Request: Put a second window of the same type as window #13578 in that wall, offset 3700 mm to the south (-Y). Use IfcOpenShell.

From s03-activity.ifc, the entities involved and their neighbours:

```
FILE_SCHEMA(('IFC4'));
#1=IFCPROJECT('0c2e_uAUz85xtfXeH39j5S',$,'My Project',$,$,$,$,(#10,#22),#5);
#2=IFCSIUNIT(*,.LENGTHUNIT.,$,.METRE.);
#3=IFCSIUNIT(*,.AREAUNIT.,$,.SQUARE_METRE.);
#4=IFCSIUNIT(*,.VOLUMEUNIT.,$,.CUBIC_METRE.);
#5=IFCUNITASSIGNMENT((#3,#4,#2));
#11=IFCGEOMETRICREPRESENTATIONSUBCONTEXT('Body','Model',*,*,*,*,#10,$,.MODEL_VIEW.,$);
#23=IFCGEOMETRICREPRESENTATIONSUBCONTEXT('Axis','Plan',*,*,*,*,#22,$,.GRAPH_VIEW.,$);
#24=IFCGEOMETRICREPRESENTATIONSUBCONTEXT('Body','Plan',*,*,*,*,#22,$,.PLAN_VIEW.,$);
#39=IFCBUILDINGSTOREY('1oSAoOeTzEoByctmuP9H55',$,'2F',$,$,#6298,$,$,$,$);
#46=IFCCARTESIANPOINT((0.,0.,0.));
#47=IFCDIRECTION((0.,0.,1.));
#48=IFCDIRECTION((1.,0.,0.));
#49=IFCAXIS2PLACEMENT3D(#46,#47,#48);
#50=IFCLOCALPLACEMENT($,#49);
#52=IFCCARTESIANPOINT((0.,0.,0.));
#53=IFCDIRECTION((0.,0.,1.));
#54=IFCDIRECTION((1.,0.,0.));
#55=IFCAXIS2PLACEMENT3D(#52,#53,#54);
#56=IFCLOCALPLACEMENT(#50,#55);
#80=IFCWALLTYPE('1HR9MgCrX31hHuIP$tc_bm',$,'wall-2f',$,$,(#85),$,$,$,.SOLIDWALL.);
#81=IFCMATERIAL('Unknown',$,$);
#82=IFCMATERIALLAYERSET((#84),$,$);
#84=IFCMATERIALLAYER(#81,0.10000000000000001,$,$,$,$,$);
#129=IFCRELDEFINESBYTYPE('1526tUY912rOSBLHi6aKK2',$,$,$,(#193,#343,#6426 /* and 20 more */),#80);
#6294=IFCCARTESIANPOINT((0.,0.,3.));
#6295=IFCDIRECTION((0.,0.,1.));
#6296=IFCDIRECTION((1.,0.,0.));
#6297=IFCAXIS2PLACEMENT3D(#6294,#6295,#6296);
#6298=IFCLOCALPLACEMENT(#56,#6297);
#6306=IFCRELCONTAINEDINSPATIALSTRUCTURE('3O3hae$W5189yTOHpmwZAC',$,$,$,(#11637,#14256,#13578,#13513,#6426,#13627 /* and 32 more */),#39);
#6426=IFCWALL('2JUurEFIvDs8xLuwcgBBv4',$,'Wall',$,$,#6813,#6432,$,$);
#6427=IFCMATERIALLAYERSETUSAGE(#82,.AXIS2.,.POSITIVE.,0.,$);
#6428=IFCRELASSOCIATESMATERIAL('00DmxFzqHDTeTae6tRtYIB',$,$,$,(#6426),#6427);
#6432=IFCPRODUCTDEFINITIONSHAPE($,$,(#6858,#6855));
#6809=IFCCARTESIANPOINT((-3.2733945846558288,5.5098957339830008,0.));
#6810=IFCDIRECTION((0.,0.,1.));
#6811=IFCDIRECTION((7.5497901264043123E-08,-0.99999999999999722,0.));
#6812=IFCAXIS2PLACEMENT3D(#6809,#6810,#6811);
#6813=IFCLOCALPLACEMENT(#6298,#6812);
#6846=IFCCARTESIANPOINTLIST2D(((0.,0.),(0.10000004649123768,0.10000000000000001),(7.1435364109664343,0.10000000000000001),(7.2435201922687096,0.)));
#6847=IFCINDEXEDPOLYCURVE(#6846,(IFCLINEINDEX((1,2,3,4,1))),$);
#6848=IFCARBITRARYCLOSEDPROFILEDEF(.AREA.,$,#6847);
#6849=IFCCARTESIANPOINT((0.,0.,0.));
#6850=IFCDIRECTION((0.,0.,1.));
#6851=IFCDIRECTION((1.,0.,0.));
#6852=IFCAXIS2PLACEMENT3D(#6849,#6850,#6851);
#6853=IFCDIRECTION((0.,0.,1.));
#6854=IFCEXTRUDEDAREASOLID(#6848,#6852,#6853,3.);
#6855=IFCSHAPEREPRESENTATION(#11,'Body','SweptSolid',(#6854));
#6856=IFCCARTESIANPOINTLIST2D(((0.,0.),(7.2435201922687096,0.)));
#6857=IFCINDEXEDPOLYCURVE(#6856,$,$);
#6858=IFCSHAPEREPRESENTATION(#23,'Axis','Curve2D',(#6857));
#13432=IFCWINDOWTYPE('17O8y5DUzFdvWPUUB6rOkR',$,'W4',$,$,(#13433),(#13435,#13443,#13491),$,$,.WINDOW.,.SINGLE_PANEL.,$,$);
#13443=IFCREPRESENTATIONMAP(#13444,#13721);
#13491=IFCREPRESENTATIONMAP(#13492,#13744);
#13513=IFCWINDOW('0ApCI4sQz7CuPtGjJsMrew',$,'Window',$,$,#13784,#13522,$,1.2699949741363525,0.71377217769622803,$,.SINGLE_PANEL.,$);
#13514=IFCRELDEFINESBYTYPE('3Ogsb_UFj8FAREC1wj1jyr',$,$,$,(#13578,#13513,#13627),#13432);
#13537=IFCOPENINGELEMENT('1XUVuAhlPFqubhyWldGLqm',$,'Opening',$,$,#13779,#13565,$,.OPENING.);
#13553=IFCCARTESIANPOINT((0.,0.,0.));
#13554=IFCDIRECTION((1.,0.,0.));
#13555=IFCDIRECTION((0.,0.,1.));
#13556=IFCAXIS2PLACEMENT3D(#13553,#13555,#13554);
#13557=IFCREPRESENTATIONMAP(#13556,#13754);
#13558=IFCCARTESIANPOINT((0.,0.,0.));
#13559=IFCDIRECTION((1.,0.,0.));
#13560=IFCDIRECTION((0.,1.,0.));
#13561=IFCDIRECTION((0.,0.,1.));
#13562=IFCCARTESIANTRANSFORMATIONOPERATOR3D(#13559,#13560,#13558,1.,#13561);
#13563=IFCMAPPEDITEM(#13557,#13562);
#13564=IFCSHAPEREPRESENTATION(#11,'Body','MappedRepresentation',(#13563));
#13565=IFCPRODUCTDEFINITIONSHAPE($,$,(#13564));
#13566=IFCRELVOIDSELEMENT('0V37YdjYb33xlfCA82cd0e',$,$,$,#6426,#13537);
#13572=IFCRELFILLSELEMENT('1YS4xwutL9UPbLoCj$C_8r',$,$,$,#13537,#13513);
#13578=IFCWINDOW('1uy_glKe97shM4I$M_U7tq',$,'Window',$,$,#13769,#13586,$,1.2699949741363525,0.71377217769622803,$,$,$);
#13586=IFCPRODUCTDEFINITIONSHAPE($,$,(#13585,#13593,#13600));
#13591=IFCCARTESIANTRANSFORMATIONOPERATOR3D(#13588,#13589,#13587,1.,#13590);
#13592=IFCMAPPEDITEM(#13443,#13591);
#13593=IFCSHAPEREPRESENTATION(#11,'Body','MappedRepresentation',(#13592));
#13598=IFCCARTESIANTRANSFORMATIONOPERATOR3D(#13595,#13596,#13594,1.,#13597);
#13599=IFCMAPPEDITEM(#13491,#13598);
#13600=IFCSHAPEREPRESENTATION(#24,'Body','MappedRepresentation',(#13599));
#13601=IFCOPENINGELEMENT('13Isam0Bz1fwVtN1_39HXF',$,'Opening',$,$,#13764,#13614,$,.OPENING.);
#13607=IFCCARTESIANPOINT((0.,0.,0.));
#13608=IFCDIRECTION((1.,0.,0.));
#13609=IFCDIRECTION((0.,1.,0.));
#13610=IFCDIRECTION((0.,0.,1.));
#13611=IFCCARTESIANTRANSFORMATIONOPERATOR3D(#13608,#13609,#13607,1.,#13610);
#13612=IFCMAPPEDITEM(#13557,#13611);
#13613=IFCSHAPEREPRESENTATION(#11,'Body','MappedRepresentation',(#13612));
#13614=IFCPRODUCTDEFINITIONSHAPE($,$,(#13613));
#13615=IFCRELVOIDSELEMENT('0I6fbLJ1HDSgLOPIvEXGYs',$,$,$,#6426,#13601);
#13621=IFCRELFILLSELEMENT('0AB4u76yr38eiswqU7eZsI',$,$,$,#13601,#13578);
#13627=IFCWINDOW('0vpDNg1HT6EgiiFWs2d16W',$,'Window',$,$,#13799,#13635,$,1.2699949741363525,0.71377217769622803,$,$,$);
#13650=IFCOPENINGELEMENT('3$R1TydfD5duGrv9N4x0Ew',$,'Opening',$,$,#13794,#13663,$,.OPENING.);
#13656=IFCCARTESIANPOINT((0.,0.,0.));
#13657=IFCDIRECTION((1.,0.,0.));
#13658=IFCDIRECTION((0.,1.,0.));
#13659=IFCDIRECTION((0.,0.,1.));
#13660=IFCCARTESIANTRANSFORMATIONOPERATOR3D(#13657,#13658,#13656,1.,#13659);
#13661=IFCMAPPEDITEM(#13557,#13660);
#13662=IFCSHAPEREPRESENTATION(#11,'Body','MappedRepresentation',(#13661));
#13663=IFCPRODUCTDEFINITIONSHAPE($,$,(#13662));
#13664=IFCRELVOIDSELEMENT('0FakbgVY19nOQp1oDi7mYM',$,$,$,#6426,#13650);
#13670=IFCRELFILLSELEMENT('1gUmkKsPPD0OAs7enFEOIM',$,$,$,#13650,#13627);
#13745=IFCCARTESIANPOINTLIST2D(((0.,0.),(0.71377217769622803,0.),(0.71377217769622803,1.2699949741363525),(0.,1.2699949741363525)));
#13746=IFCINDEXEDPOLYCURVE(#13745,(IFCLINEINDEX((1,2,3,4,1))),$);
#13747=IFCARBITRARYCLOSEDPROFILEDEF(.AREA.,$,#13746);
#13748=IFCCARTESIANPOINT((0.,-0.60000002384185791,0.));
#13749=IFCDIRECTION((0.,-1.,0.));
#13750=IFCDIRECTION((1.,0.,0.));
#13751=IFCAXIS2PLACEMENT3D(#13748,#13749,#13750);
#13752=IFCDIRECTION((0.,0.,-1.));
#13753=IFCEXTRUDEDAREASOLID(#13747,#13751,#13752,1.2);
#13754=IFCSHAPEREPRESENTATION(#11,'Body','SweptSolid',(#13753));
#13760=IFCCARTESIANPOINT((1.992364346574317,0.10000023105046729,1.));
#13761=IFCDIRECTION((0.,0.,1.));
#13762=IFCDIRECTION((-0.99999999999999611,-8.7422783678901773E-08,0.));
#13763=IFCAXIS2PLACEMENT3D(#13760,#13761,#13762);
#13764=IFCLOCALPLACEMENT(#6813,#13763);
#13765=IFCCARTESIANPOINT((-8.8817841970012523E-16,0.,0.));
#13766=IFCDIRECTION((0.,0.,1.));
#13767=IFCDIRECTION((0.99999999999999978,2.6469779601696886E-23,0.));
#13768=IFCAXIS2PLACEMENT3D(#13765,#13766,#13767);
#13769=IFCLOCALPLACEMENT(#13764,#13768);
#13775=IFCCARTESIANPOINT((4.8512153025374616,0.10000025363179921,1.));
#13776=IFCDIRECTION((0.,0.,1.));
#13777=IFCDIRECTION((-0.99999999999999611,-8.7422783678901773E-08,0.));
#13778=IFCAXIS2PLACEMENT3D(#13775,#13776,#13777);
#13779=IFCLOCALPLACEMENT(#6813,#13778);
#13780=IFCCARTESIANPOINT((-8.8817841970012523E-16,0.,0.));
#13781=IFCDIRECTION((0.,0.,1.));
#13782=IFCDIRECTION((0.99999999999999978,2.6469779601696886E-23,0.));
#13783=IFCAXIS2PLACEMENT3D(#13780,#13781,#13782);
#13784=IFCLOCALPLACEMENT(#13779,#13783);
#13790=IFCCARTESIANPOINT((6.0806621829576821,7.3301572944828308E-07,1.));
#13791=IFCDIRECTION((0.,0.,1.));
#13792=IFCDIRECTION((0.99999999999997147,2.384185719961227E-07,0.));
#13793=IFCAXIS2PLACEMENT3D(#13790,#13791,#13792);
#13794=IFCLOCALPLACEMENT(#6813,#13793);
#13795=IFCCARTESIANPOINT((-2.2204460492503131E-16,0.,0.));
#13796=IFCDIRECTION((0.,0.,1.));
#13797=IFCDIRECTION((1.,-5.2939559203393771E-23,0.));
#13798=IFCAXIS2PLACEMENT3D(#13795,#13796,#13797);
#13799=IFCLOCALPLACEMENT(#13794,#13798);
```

```python
import ifcopenshell
import ifcopenshell.api.feature
import ifcopenshell.api.geometry
import ifcopenshell.api.root
import ifcopenshell.geom
import ifcopenshell.util.element
import ifcopenshell.util.placement
import ifcopenshell.util.shape

model = ifcopenshell.open("s03-activity.ifc")
settings = ifcopenshell.geom.settings()


def volume(element):
    """Net volume in cubic metres, openings subtracted."""
    shape = ifcopenshell.geom.create_shape(settings, element)
    return ifcopenshell.util.shape.get_volume(shape.geometry)


window = model.by_id(13578)
opening = window.FillsVoids[0].RelatingOpeningElement
wall = opening.VoidsElements[0].RelatingBuildingElement
before = volume(wall)
shift = ifcopenshell.util.placement.get_local_placement(wall.ObjectPlacement)[:3, 0] * 3.7

# copy_class copies the void relationship, type, container and properties, but no geometry.
new_opening = ifcopenshell.api.root.copy_class(model, product=opening)
new_opening.Representation = ifcopenshell.util.element.copy_deep(
    model, opening.Representation, exclude=["IfcGeometricRepresentationContext", "IfcRepresentationMap"]
)
new_window = ifcopenshell.api.root.copy_class(model, product=window)
new_window.Representation = ifcopenshell.util.element.copy_deep(
    model, window.Representation, exclude=["IfcGeometricRepresentationContext", "IfcRepresentationMap"]
)
ifcopenshell.api.feature.add_filling(model, opening=new_opening, element=new_window)

for old, new in ((opening, new_opening), (window, new_window)):
    matrix = ifcopenshell.util.placement.get_local_placement(old.ObjectPlacement)
    matrix[:3, 3] += shift
    ifcopenshell.api.geometry.edit_object_placement(model, product=new, matrix=matrix, is_si=False)

after = volume(wall)

print(f"wall volume {before:.3f} -> {after:.3f} m3")

model.write("s03-activity_edited.ifc")
```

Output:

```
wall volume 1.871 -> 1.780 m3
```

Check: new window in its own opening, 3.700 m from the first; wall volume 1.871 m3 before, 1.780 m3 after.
